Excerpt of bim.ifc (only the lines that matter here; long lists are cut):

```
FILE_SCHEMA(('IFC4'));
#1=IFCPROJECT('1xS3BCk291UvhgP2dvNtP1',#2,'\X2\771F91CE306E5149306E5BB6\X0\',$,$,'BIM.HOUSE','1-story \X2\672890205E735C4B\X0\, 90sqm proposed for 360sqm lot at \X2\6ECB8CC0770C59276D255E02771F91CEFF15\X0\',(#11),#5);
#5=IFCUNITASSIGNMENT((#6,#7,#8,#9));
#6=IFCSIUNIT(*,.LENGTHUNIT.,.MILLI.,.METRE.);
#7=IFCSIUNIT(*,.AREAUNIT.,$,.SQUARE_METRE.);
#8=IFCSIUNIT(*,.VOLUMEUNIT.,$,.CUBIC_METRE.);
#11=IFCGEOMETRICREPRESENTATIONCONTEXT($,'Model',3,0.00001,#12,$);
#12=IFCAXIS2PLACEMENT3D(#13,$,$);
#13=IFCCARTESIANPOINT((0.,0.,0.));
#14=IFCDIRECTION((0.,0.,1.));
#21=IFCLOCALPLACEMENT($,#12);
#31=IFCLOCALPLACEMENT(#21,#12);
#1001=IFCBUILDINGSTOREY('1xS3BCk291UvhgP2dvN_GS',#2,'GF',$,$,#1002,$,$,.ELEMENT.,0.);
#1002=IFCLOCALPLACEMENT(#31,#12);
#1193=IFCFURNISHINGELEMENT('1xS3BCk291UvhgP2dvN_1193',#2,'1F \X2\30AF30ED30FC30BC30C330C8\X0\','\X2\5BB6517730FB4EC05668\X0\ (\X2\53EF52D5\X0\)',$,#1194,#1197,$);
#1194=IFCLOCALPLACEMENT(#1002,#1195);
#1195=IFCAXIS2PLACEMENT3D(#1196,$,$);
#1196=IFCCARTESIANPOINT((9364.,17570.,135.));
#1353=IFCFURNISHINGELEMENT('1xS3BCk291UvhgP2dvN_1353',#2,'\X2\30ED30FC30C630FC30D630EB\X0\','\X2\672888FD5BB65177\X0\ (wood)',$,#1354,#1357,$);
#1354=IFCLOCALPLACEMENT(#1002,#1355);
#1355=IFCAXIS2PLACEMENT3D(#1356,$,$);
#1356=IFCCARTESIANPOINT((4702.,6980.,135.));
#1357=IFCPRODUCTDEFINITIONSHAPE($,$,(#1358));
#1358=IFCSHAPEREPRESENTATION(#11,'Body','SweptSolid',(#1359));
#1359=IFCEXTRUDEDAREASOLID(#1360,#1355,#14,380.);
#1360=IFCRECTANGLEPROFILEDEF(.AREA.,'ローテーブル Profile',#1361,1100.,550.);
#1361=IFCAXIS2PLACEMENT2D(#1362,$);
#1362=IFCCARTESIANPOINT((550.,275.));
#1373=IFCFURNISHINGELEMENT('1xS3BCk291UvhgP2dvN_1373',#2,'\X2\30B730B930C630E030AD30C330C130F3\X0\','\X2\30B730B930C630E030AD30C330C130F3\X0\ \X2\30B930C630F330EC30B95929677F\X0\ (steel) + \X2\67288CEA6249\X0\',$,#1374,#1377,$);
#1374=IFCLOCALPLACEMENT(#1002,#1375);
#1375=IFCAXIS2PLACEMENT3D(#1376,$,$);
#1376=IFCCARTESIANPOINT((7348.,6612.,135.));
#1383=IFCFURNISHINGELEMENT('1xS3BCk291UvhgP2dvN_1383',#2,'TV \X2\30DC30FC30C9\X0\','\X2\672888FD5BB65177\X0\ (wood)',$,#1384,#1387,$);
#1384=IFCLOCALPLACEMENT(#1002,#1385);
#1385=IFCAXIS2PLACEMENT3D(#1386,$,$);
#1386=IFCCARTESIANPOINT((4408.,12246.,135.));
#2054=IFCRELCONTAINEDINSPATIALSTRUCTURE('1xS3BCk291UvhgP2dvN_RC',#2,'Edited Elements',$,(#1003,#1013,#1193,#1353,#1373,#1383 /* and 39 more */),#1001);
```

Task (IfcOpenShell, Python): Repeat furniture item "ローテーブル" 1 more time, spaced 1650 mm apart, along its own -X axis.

```python
import ifcopenshell
import ifcopenshell.api.geometry
import ifcopenshell.api.root
import ifcopenshell.util.element
import ifcopenshell.util.placement
import ifcopenshell.util.unit

model = ifcopenshell.open("bim.ifc")
unit_scale = ifcopenshell.util.unit.calculate_unit_scale(model)


def reuse_history(source, copy):
    """copy_class also copies each property set's owner history, people and application; keep the originals."""
    for rel in copy.IsDefinedBy:
        if rel.is_a("IfcRelDefinesByProperties") and (history := rel.RelatingPropertyDefinition.OwnerHistory):
            rel.RelatingPropertyDefinition.OwnerHistory = source.OwnerHistory
            ifcopenshell.util.element.remove_deep2(model, history)


source = model.by_guid("1xS3BCk291UvhgP2dvN_1353")
base = ifcopenshell.util.placement.get_local_placement(source.ObjectPlacement)
step = -base[:3, 0] * 1.65 / unit_scale

for i in range(1, 2):
    copy = ifcopenshell.api.root.copy_class(model, product=source)
    copy.Representation = ifcopenshell.util.element.copy_deep(
        model, source.Representation, exclude=["IfcGeometricRepresentationContext", "IfcRepresentationMap"]
    )
    reuse_history(source, copy)
    matrix = base.copy()
    matrix[:3, 3] += i * step
    print("added at", matrix[:3, 3].round(3) + 0.0)
    ifcopenshell.api.geometry.edit_object_placement(model, product=copy, matrix=matrix, is_si=False)

model.write("bim_edited.ifc")
```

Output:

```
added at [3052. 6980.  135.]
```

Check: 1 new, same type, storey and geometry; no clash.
